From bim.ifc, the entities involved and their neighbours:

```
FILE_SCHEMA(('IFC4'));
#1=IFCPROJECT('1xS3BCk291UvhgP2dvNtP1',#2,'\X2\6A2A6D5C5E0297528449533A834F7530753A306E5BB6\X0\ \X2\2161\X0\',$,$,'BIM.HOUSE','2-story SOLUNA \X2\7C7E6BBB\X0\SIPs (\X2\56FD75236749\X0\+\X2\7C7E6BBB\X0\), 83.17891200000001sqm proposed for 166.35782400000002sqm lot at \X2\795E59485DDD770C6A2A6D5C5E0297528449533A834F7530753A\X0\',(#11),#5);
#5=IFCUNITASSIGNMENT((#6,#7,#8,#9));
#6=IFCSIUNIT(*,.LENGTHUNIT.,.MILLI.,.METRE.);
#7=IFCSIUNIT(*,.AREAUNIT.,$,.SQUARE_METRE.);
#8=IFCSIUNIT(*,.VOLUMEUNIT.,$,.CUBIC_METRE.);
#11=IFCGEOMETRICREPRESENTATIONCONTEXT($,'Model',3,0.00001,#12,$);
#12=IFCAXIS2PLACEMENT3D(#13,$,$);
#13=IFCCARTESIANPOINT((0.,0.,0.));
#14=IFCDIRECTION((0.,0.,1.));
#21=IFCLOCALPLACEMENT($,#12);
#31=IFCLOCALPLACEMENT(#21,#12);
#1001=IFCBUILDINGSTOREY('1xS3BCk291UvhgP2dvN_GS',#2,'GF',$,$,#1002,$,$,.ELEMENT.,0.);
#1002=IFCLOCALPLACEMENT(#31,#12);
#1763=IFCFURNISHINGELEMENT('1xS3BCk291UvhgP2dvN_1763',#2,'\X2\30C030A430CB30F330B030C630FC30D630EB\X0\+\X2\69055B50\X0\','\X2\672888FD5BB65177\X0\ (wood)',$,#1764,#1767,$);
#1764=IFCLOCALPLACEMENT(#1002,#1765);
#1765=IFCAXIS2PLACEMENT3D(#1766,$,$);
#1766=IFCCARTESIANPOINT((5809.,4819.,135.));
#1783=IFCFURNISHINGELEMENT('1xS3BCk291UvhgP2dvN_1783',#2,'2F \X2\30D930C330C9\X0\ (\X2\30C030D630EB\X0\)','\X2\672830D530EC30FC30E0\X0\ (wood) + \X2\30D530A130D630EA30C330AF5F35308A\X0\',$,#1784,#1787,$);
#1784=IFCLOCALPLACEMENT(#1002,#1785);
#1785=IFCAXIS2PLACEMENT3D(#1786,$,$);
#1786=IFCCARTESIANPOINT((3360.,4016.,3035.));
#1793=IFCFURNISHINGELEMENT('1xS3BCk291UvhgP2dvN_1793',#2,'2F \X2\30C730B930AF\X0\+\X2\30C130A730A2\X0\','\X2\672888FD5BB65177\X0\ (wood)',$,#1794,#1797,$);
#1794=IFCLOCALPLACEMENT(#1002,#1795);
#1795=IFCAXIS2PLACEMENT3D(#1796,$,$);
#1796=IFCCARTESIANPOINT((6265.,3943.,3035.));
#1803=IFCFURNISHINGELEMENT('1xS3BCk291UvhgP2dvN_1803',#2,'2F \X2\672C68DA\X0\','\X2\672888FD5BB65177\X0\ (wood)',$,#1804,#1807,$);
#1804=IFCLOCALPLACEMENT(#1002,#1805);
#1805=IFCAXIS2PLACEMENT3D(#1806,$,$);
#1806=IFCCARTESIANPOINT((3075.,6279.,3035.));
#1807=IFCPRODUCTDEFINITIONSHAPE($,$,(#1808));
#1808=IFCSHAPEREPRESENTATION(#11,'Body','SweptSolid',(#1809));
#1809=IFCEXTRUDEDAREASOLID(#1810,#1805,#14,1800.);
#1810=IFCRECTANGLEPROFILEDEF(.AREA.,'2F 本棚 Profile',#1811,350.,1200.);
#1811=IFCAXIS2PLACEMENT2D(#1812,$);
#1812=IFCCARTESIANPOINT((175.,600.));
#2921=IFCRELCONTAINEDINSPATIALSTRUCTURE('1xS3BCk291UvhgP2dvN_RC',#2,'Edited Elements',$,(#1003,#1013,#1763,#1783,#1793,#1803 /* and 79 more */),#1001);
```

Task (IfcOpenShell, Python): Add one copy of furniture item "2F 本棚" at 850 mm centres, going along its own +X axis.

```python
import ifcopenshell
import ifcopenshell.api.geometry
import ifcopenshell.api.root
import ifcopenshell.util.element
import ifcopenshell.util.placement

model = ifcopenshell.open("bim.ifc")


def reuse_history(source, copy):
    """copy_class also copies each property set's owner history, people and application; keep the originals."""
    for rel in copy.IsDefinedBy:
        if rel.is_a("IfcRelDefinesByProperties") and (history := rel.RelatingPropertyDefinition.OwnerHistory):
            rel.RelatingPropertyDefinition.OwnerHistory = source.OwnerHistory
            ifcopenshell.util.element.remove_deep2(model, history)


source = model.by_guid("1xS3BCk291UvhgP2dvN_1803")
base = ifcopenshell.util.placement.get_local_placement(source.ObjectPlacement)
step = base[:3, 0] * 850.0

for i in range(1, 2):
    copy = ifcopenshell.api.root.copy_class(model, product=source)
    copy.Representation = ifcopenshell.util.element.copy_deep(
        model, source.Representation, exclude=["IfcGeometricRepresentationContext", "IfcRepresentationMap"]
    )
    reuse_history(source, copy)
    matrix = base.copy()
    matrix[:3, 3] += i * step
    print("added at", matrix[:3, 3].round(3) + 0.0)
    ifcopenshell.api.geometry.edit_object_placement(model, product=copy, matrix=matrix, is_si=False)

model.write("bim_rev.ifc")
```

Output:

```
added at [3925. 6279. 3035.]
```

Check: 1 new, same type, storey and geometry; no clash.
